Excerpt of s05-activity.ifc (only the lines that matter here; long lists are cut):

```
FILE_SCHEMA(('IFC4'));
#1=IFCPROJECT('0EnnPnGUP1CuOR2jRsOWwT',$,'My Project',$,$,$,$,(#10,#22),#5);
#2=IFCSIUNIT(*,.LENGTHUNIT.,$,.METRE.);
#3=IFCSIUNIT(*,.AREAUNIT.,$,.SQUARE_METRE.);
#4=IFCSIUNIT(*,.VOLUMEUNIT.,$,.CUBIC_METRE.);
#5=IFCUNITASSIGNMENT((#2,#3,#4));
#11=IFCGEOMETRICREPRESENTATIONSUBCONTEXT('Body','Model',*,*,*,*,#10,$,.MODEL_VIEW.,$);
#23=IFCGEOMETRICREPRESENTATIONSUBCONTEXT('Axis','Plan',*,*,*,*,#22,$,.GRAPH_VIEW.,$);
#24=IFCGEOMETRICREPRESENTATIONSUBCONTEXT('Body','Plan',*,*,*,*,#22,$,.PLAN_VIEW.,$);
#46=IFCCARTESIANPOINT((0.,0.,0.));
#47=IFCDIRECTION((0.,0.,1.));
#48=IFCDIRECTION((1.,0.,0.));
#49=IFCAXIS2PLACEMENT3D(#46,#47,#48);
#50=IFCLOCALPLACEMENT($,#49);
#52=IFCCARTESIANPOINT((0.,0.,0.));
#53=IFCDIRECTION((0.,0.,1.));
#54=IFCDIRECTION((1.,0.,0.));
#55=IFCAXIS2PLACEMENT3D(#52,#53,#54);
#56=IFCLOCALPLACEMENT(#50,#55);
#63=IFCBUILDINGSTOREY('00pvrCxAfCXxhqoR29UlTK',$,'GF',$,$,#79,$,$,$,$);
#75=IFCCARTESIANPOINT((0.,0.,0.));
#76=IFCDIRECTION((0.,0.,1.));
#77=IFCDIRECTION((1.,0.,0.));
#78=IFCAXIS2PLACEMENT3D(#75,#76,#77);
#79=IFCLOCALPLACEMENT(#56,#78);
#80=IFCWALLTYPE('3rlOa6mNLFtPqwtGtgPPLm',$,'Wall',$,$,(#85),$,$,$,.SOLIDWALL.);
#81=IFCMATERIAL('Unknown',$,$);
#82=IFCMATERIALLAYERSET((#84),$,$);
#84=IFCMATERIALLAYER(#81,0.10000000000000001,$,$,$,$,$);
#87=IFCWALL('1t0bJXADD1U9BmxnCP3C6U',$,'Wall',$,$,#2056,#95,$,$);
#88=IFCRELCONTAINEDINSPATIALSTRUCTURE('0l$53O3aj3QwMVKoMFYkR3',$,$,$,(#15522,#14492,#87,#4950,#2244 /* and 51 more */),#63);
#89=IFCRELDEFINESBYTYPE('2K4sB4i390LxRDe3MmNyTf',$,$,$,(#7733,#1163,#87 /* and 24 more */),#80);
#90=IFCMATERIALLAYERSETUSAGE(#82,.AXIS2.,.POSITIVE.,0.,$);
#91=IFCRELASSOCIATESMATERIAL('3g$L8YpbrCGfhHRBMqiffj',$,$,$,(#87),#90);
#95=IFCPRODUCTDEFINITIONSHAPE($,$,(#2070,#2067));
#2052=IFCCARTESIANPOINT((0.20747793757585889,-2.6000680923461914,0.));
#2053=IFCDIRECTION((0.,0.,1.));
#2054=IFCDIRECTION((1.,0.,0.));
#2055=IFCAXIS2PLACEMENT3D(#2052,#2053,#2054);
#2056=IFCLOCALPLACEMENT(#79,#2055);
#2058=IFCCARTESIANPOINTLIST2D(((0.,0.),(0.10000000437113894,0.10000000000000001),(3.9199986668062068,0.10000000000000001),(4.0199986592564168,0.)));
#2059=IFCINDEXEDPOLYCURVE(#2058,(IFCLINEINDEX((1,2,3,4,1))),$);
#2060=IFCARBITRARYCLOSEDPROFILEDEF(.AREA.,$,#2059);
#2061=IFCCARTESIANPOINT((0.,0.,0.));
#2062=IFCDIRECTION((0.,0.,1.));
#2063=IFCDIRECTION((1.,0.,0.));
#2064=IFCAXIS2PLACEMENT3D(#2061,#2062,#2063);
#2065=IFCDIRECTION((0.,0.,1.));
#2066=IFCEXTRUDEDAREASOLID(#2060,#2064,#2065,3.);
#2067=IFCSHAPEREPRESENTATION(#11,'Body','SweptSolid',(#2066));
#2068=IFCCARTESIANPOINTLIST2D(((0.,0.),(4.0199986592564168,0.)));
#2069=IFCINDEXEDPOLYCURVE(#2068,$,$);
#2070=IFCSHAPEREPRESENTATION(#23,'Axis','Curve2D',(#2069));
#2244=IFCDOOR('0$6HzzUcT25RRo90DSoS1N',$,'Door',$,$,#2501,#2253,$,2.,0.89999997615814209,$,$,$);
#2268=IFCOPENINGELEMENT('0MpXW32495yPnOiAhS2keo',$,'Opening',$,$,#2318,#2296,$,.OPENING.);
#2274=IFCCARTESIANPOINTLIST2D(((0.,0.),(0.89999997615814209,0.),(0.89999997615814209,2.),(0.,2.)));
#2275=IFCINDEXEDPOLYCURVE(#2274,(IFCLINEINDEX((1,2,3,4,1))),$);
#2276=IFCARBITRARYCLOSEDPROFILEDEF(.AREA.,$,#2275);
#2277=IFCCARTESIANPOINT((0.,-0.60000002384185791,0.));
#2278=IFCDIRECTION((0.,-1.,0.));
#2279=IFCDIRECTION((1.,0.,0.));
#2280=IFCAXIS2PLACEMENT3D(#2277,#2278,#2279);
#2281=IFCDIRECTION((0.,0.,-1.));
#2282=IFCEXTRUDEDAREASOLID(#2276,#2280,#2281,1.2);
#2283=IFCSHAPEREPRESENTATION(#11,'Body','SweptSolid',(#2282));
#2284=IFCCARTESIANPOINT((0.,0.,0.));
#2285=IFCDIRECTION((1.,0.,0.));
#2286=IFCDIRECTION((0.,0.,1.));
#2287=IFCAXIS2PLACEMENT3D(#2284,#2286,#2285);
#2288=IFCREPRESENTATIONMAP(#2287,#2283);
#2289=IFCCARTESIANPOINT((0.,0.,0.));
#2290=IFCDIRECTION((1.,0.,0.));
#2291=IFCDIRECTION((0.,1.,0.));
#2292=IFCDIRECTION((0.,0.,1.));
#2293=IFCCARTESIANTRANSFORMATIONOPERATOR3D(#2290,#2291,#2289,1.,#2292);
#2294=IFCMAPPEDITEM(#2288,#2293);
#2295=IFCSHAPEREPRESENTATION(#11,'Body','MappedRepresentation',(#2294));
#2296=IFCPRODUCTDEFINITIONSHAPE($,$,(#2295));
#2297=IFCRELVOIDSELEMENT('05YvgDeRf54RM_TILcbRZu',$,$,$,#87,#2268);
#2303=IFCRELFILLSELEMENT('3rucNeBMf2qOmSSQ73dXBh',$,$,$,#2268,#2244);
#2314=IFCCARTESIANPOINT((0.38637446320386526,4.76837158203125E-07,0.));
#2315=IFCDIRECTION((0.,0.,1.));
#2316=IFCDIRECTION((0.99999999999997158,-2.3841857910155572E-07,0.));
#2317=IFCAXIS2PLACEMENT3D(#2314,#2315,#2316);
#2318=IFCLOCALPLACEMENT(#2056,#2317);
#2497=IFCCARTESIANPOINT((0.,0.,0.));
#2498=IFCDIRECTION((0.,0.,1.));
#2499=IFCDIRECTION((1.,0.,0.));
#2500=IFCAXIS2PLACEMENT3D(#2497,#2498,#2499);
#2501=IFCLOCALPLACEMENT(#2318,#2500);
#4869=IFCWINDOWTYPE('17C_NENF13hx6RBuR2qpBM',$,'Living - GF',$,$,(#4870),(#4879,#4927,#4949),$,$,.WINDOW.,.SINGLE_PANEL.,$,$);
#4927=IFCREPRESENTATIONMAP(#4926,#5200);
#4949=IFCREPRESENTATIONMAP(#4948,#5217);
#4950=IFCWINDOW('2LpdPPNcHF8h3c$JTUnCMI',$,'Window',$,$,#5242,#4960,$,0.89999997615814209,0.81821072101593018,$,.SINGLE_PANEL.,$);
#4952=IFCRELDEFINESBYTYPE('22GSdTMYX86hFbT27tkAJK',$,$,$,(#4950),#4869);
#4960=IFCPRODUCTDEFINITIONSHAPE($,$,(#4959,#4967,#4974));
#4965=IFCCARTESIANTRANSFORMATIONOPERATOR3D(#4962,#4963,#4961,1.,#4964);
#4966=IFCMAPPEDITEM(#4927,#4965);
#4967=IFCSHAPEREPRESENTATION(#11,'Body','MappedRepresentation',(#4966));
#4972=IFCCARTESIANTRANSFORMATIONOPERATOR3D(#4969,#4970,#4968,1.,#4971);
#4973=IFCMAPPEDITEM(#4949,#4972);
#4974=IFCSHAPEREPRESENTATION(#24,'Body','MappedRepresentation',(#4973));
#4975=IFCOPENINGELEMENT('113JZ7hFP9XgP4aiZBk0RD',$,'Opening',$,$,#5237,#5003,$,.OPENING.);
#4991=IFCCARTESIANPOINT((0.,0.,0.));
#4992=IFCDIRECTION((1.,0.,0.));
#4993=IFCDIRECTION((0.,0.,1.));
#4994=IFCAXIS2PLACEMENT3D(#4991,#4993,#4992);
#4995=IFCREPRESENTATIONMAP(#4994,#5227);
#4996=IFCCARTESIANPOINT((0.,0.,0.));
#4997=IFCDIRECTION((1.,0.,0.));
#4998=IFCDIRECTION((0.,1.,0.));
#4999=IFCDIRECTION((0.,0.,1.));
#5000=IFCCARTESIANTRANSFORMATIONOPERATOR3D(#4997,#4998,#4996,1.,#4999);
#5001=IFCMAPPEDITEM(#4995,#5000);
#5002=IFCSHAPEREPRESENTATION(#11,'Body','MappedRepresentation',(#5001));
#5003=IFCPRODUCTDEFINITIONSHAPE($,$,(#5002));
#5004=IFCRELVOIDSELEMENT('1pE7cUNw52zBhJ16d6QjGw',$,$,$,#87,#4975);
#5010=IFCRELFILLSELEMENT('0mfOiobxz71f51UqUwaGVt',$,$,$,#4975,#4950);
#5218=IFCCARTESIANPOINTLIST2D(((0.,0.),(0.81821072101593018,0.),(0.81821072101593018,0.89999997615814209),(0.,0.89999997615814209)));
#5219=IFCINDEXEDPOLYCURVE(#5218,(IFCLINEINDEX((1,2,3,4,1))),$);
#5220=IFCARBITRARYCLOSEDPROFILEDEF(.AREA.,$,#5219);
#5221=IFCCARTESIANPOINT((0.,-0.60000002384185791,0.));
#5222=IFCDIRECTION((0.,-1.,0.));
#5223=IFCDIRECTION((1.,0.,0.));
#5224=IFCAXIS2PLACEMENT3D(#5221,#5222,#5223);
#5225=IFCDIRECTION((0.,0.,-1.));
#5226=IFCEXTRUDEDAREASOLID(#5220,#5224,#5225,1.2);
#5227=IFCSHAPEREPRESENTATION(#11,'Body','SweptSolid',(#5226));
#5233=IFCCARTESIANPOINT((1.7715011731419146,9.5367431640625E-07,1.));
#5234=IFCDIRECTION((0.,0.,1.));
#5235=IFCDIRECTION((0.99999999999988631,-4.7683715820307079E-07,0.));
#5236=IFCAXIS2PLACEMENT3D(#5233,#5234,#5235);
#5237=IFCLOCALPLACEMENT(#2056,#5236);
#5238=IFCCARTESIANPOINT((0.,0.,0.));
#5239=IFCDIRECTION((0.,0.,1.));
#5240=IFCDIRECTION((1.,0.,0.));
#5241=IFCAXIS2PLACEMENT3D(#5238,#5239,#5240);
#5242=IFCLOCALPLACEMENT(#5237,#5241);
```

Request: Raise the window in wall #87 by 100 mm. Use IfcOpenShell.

```python
import numpy as np
import ifcopenshell
import ifcopenshell.api.geometry
import ifcopenshell.util.placement
import ifcopenshell.util.unit

model = ifcopenshell.open("s05-activity.ifc")
unit_scale = ifcopenshell.util.unit.calculate_unit_scale(model)

window = model.by_guid("2LpdPPNcHF8h3c$JTUnCMI")
opening = window.FillsVoids[0].RelatingOpeningElement
dz = 0.1 / unit_scale

shift = np.array([0.0, 0.0, dz])
# The window is placed relative to its opening, so it follows when the opening moves.
matrix = ifcopenshell.util.placement.get_local_placement(opening.ObjectPlacement)
matrix[:3, 3] += shift
ifcopenshell.api.geometry.edit_object_placement(
    model, product=opening, matrix=matrix, is_si=False, should_transform_children=True
)

print(f"moved by {dz * unit_scale:+.3f} m")

model.write("s05-activity_edited.ifc")
```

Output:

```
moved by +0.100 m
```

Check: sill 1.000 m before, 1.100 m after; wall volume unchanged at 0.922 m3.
